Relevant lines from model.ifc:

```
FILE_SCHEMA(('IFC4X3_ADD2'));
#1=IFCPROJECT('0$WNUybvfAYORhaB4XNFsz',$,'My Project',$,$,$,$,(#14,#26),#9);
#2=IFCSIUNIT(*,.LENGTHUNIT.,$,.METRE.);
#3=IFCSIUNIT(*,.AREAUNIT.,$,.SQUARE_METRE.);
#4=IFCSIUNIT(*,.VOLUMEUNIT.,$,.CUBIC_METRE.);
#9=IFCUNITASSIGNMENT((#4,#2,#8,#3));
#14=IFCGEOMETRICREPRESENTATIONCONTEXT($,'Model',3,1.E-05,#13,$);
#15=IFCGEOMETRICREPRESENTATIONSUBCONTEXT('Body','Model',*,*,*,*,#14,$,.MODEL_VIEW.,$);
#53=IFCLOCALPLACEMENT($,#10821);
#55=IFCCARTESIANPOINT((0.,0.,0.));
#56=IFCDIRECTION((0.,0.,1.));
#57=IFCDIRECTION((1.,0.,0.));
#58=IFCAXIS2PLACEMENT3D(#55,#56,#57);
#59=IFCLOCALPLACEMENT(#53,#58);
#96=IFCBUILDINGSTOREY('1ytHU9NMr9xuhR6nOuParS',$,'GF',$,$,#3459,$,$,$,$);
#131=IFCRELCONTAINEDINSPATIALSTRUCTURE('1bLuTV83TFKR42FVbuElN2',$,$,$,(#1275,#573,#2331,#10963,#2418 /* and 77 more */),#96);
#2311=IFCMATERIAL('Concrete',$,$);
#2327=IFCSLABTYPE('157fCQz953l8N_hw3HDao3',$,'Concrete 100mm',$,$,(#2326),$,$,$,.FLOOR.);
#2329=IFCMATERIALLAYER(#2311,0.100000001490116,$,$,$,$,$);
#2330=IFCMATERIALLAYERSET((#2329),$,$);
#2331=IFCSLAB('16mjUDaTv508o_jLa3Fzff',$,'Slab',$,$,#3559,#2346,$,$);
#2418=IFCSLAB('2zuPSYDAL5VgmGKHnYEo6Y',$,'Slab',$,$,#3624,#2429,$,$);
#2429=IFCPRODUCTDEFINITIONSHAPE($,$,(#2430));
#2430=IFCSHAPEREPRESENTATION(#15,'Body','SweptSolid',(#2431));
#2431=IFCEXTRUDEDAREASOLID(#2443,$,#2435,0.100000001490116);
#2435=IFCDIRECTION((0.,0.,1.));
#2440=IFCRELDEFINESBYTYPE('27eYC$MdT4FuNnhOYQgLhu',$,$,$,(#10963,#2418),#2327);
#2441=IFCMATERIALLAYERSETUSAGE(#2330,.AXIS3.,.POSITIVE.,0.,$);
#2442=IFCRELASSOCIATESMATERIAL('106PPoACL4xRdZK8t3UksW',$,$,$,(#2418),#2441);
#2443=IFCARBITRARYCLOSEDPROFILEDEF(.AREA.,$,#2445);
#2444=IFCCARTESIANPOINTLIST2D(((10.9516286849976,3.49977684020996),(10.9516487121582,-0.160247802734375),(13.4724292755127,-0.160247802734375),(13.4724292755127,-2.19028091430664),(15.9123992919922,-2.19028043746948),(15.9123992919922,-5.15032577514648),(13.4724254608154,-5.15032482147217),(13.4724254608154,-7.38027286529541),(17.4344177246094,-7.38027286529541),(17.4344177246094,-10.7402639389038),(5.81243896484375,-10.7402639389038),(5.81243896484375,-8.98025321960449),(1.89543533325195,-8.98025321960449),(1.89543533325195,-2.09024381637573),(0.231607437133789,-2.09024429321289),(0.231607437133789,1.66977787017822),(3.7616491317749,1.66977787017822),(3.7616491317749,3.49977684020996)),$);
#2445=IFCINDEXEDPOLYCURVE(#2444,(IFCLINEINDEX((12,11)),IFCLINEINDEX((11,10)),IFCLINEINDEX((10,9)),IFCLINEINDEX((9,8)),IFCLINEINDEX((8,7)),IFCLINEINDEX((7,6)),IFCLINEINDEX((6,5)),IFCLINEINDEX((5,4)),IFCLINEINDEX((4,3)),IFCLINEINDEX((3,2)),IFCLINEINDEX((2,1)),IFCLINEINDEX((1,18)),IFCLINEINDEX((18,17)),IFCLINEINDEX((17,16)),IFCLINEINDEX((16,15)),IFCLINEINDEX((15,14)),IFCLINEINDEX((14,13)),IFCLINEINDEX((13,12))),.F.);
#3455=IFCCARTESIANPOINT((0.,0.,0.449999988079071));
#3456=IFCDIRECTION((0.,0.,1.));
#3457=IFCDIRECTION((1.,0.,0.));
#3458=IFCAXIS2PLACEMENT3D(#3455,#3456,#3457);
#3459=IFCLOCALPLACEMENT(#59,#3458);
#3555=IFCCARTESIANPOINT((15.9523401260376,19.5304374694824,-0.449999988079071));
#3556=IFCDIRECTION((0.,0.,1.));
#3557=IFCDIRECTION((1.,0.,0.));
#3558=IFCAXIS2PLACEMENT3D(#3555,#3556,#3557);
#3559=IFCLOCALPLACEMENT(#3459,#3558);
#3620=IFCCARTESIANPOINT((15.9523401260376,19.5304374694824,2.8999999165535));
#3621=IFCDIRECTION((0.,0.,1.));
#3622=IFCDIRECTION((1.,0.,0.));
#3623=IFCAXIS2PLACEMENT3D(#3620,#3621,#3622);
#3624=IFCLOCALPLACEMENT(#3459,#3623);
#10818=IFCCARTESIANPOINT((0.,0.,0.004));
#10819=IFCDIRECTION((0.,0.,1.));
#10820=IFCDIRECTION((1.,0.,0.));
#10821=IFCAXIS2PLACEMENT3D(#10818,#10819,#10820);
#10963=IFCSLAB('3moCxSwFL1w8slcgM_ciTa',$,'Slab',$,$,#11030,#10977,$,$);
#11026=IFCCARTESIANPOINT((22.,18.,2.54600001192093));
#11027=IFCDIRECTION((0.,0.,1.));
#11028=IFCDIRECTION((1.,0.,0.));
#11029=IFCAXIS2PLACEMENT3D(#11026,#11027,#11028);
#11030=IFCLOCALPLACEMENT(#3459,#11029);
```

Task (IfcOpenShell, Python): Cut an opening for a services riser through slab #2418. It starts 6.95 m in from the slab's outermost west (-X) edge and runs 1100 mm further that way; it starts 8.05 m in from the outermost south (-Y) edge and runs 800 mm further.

```python
import numpy as np
import ifcopenshell
import ifcopenshell.api.feature
import ifcopenshell.api.geometry
import ifcopenshell.api.root
import ifcopenshell.geom
import ifcopenshell.util.placement
import ifcopenshell.util.representation
import ifcopenshell.util.shape
import ifcopenshell.util.unit

model = ifcopenshell.open("model.ifc")
unit_scale = ifcopenshell.util.unit.calculate_unit_scale(model)
settings = ifcopenshell.geom.settings()


def volume(element):
    """Net volume in cubic metres, openings subtracted."""
    shape = ifcopenshell.geom.create_shape(settings, element)
    return ifcopenshell.util.shape.get_volume(shape.geometry)


slab = model.by_guid("2zuPSYDAL5VgmGKHnYEo6Y")
before = volume(slab)

# Extent in the slab's own axes, in metres. The edges named are its -X and -Y sides.
slab_shape = ifcopenshell.geom.create_shape(settings, slab)
vertices = ifcopenshell.util.shape.get_vertices(slab_shape.geometry)
x_min, y_min, bottom = vertices.min(axis=0)
top = vertices[:, 2].max()

opening = ifcopenshell.api.root.create_entity(model, ifc_class="IfcOpeningElement", name="Services riser opening", predefined_type="OPENING")
context = ifcopenshell.util.representation.get_context(model, "Model", "Body", "MODEL_VIEW")
width, depth = 1.1, 0.8
outline = [(0.0, 0.0), (width, 0.0), (width, depth), (0.0, depth), (0.0, 0.0)]
# Overshoot both faces by 50 mm so the cut is clean.
shape = ifcopenshell.api.geometry.add_slab_representation(
    model, context=context, depth=top - bottom + 0.1, polyline=outline
)
ifcopenshell.api.geometry.assign_representation(model, product=opening, representation=shape)

matrix = ifcopenshell.util.placement.get_local_placement(slab.ObjectPlacement)
matrix[:, 3] = matrix @ np.append(np.array([x_min + 6.95, y_min + 8.05, bottom - 0.05]) / unit_scale, 1.0)
ifcopenshell.api.geometry.edit_object_placement(model, product=opening, matrix=matrix, is_si=False)
ifcopenshell.api.feature.add_feature(model, feature=opening, element=slab)

after = volume(slab)

print(f"slab volume {before:.3f} -> {after:.3f} m3")

model.write("model_edited.ifc")
```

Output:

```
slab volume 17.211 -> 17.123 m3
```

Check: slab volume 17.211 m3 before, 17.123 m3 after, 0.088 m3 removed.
